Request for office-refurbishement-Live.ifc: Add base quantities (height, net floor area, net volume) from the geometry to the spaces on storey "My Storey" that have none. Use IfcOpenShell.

First a look at what the model holds.

```python
import ifcopenshell
import ifcopenshell.util.element
import ifcopenshell.util.unit

model = ifcopenshell.open("office-refurbishement-Live.ifc")
print(model.schema)
for unit_type in ("LENGTHUNIT", "AREAUNIT", "VOLUMEUNIT"):
    print(unit_type, ifcopenshell.util.unit.calculate_unit_scale(model, unit_type))
storey = next(s for s in model.by_type("IfcBuildingStorey") if s.Name == "My Storey")
spaces = [e for e in ifcopenshell.util.element.get_decomposition(storey) if e.is_a("IfcSpace")]
for e in sorted(spaces, key=lambda e: e.id()):
    print(e.id(), e.is_a(), e.Name, list(ifcopenshell.util.element.get_psets(e, qtos_only=True)), sep=" | ")
```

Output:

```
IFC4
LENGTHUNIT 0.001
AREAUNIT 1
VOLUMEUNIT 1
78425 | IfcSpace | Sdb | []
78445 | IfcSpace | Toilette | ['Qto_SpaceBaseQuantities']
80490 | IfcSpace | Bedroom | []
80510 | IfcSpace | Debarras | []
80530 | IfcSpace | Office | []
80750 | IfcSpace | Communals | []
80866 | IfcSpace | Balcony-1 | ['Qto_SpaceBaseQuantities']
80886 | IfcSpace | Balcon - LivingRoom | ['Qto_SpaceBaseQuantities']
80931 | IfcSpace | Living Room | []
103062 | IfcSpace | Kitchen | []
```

```python
import ifcopenshell
import ifcopenshell.api.pset
import ifcopenshell.geom
import ifcopenshell.util.element
import ifcopenshell.util.shape
import ifcopenshell.util.unit

model = ifcopenshell.open("office-refurbishement-Live.ifc")
unit_scale = ifcopenshell.util.unit.calculate_unit_scale(model)
area_scale = ifcopenshell.util.unit.calculate_unit_scale(model, "AREAUNIT")
volume_scale = ifcopenshell.util.unit.calculate_unit_scale(model, "VOLUMEUNIT")
settings = ifcopenshell.geom.settings()

storey = next(s for s in model.by_type("IfcBuildingStorey") if s.Name == "My Storey")
spaces = [e for e in ifcopenshell.util.element.get_decomposition(storey) if e.is_a("IfcSpace")]

for e in sorted(spaces, key=lambda e: e.id()):
    if ifcopenshell.util.element.get_psets(e, qtos_only=True, should_inherit=False):
        continue
    # Geometry comes back in metres, in the element's own axes.
    shape = ifcopenshell.geom.create_shape(settings, e)
    values = {
        "Height": ifcopenshell.util.shape.get_z(shape.geometry) / unit_scale,
        "NetFloorArea": ifcopenshell.util.shape.get_footprint_area(shape.geometry) / area_scale,
        "NetVolume": ifcopenshell.util.shape.get_volume(shape.geometry) / volume_scale,
    }
    qto = ifcopenshell.api.pset.add_qto(model, product=e, name="Qto_SpaceBaseQuantities")
    ifcopenshell.api.pset.edit_qto(model, qto=qto, properties=values)
    print(e.id(), {k: round(v, 3) for k, v in values.items()})

model.write("office-refurbishement-Live-out.ifc")
```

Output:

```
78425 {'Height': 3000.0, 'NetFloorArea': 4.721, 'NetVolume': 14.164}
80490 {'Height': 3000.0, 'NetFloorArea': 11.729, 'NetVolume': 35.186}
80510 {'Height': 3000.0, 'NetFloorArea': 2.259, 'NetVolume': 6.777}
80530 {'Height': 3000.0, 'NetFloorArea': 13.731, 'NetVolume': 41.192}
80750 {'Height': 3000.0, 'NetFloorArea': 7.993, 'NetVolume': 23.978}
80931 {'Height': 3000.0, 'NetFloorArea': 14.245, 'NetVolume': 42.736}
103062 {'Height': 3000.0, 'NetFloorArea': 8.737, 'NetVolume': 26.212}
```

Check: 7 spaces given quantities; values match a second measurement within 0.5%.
